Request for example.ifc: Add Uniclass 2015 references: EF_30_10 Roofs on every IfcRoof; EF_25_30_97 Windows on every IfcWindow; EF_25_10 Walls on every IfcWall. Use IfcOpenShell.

First a look at what the model holds.

```python
import ifcopenshell

model = ifcopenshell.open("example.ifc")
print(model.schema)
print("classifications:", [c.Name for c in model.by_type("IfcClassification")])
for ifc_class in ("IfcDoor", "IfcRoof", "IfcStair", "IfcWall", "IfcWindow"):
    print(ifc_class, len(model.by_type(ifc_class)))
```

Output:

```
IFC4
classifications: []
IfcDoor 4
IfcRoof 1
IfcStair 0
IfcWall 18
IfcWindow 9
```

```python
import ifcopenshell
import ifcopenshell.api.classification

model = ifcopenshell.open("example.ifc")

system = ifcopenshell.api.classification.add_classification(model, classification="Uniclass 2015")

codes = {
    "IfcRoof": ("EF_30_10", "Roofs"),
    "IfcWindow": ("EF_25_30_97", "Windows"),
    "IfcWall": ("EF_25_10", "Walls"),
}
for ifc_class, (code, name) in codes.items():
    products = model.by_type(ifc_class)
    ifcopenshell.api.classification.add_reference(
        model, products=products, classification=system, identification=code, name=name
    )
    print(code, len(products))

model.write("example_edited.ifc")
```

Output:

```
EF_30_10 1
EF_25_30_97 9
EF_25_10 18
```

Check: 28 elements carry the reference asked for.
